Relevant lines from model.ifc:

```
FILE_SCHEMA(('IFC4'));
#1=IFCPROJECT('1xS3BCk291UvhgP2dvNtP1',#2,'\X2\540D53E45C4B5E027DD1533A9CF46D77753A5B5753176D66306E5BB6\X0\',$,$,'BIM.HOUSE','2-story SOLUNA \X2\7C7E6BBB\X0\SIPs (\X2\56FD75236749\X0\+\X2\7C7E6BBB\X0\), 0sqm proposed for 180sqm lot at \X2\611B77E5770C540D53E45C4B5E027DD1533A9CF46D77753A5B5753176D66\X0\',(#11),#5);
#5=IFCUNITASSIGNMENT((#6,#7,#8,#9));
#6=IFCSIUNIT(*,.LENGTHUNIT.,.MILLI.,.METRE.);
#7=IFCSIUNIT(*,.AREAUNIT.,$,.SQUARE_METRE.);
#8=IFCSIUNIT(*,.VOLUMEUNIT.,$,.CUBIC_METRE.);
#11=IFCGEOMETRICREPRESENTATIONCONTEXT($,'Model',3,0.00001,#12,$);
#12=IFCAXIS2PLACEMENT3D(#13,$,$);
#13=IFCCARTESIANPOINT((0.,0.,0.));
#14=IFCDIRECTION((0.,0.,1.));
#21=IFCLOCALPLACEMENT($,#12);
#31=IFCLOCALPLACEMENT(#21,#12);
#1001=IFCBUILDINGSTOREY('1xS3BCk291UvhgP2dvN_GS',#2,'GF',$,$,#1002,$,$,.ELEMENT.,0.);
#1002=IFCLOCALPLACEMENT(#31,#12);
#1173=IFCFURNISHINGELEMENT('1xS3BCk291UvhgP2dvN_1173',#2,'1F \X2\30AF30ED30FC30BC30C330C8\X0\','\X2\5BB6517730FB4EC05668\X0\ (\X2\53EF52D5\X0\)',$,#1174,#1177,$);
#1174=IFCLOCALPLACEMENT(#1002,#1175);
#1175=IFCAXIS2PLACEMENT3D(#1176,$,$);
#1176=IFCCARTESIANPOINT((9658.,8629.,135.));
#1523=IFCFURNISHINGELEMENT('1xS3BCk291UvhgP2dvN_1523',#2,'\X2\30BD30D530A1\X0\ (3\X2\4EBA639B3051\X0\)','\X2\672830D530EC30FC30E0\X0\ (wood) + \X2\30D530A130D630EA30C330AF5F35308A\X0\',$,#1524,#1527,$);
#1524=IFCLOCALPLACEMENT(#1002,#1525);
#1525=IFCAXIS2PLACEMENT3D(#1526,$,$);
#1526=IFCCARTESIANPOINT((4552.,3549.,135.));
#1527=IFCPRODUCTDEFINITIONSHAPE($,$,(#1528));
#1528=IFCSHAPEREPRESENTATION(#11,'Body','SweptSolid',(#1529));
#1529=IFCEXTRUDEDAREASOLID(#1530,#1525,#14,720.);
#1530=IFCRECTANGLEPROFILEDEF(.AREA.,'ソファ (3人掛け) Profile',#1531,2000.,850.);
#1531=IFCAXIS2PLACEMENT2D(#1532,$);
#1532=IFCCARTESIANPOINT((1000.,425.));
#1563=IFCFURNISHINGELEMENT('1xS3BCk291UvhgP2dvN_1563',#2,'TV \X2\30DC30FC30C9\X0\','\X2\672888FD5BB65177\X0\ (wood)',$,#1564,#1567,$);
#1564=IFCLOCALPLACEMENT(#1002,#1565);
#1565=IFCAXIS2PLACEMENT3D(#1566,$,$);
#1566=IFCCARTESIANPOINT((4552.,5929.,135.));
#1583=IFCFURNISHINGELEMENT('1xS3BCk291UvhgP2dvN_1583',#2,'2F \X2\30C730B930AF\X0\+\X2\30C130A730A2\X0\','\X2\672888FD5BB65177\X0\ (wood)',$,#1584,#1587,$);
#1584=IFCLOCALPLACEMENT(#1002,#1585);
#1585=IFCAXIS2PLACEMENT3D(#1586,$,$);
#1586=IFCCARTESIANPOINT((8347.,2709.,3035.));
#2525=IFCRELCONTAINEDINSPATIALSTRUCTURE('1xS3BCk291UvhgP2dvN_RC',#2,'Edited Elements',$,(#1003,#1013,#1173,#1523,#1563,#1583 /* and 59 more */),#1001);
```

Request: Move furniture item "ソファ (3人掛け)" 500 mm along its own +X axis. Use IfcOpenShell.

```python
import ifcopenshell
import ifcopenshell.api.geometry
import ifcopenshell.util.placement

model = ifcopenshell.open("model.ifc")

item = model.by_guid("1xS3BCk291UvhgP2dvN_1523")
matrix = ifcopenshell.util.placement.get_local_placement(item.ObjectPlacement)
matrix[:3, 3] += matrix[:3, 0] * 500.0
ifcopenshell.api.geometry.edit_object_placement(model, product=item, matrix=matrix, is_si=False)

print(ifcopenshell.util.placement.get_local_placement(item.ObjectPlacement).round(3) + 0.0)

model.write("model_rev.ifc")
```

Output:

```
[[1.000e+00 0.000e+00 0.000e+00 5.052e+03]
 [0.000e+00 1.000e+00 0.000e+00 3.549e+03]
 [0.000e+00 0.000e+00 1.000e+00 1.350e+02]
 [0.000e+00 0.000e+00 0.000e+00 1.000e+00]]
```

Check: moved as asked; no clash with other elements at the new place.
